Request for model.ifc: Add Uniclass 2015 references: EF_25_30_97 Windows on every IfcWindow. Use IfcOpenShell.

First a look at what the model holds.

```python
import ifcopenshell

model = ifcopenshell.open("model.ifc")
print(model.schema)
print("classifications:", [c.Name for c in model.by_type("IfcClassification")])
for ifc_class in ("IfcDoor", "IfcRoof", "IfcStair", "IfcWall", "IfcWindow"):
    print(ifc_class, len(model.by_type(ifc_class)))
```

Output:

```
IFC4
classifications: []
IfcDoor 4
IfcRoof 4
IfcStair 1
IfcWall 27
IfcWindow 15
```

```python
import ifcopenshell
import ifcopenshell.api.classification

model = ifcopenshell.open("model.ifc")

system = ifcopenshell.api.classification.add_classification(model, classification="Uniclass 2015")

codes = {
    "IfcWindow": ("EF_25_30_97", "Windows"),
}
for ifc_class, (code, name) in codes.items():
    products = model.by_type(ifc_class)
    ifcopenshell.api.classification.add_reference(
        model, products=products, classification=system, identification=code, name=name
    )
    print(code, len(products))

model.write("model_v2.ifc")
```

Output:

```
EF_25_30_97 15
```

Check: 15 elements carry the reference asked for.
